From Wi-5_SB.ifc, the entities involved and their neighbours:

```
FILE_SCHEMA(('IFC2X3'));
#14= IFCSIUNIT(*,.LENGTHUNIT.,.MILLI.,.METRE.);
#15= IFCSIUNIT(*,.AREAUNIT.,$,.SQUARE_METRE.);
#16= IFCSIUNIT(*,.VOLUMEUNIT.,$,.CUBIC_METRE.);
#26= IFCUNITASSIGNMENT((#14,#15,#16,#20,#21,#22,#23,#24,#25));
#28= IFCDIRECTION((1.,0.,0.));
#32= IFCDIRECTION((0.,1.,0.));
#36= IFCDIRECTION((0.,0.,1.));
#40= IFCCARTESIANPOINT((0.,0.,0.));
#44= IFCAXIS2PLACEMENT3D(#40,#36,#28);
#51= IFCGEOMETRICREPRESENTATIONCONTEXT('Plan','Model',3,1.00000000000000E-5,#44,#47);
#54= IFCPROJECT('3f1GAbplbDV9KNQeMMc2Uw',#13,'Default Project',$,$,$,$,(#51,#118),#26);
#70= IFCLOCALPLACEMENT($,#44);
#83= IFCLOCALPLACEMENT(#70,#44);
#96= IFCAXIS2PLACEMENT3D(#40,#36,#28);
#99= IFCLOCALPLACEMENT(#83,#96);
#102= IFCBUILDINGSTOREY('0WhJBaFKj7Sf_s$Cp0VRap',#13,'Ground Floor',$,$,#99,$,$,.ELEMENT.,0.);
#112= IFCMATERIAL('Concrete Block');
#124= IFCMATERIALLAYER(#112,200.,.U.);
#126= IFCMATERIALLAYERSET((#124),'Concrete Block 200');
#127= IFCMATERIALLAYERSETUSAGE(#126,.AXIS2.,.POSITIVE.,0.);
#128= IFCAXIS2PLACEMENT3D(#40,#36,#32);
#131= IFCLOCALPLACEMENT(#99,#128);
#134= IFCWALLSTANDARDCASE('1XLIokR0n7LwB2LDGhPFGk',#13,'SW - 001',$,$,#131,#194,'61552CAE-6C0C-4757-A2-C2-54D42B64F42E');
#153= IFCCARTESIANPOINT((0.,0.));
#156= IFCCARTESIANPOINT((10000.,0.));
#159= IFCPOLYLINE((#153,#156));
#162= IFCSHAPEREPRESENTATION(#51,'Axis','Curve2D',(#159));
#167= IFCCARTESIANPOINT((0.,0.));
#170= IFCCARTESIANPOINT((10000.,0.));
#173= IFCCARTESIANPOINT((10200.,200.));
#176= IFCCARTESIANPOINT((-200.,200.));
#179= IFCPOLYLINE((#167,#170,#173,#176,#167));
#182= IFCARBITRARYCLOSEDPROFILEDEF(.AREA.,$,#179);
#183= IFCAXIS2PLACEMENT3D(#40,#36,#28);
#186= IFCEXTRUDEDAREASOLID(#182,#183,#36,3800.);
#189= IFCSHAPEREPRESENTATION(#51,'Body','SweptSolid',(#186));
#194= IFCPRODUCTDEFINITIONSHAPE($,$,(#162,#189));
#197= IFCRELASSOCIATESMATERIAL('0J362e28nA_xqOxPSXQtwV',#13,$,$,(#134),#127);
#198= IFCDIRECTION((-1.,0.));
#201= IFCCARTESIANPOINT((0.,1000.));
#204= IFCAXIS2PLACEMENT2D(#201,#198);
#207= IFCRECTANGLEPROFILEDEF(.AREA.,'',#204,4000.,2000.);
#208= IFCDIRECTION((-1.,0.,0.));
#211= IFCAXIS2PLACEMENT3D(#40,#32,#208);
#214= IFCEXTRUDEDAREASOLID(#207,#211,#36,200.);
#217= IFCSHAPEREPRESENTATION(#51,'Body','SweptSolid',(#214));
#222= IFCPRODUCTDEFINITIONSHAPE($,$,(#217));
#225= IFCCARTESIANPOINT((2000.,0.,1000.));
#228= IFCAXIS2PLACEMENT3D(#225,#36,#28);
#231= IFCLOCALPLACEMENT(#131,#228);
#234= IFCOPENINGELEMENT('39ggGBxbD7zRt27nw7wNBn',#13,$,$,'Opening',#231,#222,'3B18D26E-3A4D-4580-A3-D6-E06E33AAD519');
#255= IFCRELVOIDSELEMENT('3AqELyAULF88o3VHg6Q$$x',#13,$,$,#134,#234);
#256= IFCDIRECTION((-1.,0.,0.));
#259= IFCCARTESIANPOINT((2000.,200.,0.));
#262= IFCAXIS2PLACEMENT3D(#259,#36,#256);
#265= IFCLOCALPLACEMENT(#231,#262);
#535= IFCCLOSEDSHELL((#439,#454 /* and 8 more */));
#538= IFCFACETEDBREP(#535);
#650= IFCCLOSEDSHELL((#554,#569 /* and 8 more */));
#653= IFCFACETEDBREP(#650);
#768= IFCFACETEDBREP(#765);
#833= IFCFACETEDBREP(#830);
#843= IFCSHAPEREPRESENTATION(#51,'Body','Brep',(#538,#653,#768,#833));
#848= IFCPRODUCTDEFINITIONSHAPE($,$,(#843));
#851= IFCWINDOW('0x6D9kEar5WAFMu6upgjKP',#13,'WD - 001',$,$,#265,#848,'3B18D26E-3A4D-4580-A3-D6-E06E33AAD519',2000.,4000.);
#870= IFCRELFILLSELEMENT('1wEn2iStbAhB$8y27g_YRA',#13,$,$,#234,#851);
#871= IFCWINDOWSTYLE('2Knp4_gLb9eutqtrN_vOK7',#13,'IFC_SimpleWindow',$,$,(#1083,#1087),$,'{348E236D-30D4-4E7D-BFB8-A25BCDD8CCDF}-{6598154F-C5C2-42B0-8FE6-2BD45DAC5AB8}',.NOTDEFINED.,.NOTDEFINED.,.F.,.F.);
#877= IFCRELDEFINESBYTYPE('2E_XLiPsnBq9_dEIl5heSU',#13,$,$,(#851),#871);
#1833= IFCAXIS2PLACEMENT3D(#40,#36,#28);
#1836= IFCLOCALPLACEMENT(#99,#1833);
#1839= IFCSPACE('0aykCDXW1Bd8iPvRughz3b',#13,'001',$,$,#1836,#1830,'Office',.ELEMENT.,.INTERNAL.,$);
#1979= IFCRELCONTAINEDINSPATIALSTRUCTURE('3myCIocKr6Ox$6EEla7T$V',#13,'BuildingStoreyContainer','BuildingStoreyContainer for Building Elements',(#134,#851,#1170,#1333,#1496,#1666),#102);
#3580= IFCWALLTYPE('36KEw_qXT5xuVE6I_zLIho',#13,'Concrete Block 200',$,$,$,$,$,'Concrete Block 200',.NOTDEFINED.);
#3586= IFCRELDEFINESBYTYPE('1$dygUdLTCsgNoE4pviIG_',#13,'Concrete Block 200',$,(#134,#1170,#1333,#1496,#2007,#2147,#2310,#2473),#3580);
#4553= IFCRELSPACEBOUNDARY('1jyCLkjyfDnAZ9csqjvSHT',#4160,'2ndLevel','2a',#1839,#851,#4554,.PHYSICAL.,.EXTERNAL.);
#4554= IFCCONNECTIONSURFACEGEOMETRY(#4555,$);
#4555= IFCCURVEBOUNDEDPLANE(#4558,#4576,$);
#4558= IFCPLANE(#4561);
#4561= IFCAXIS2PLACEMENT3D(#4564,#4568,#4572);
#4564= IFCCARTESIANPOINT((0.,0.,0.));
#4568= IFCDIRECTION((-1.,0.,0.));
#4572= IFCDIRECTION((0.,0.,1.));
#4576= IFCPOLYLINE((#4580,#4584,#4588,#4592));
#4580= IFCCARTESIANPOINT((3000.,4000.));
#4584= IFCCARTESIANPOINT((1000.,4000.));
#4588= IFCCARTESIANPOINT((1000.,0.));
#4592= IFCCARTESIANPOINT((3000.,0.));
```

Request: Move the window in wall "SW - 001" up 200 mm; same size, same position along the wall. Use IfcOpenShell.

```python
import numpy as np
import ifcopenshell
import ifcopenshell.api.geometry
import ifcopenshell.util.placement
import ifcopenshell.util.unit

model = ifcopenshell.open("Wi-5_SB.ifc")
unit_scale = ifcopenshell.util.unit.calculate_unit_scale(model)

window = model.by_guid("0x6D9kEar5WAFMu6upgjKP")
opening = window.FillsVoids[0].RelatingOpeningElement
dz = 0.2 / unit_scale

shift = np.array([0.0, 0.0, dz])
# The window is placed relative to its opening, so it follows when the opening moves.
matrix = ifcopenshell.util.placement.get_local_placement(opening.ObjectPlacement)
matrix[:3, 3] += shift
ifcopenshell.api.geometry.edit_object_placement(
    model, product=opening, matrix=matrix, is_si=False, should_transform_children=True
)

# Space boundary surfaces are stored in each space's coordinates; move them too.
for rel in window.ProvidesBoundaries:
    if not rel.ConnectionGeometry:
        continue
    surface = rel.ConnectionGeometry.SurfaceOnRelatingElement.BasisSurface
    space_matrix = ifcopenshell.util.placement.get_local_placement(rel.RelatingSpace.ObjectPlacement)
    point = np.array(surface.Position.Location.Coordinates) + space_matrix[:3, :3].T @ shift
    surface.Position = model.createIfcAxis2Placement3D(
        model.createIfcCartesianPoint(point.tolist()), surface.Position.Axis, surface.Position.RefDirection
    )

print(f"moved by {dz * unit_scale:+.3f} m")

model.write("Wi-5_SB_rev.ifc")
```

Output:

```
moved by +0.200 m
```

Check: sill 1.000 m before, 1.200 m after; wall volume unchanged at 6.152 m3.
